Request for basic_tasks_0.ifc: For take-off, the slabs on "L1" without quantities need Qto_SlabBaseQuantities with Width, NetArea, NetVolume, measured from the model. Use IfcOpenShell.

First a look at what the model holds.

```python
import ifcopenshell
import ifcopenshell.util.element
import ifcopenshell.util.unit

model = ifcopenshell.open("basic_tasks_0.ifc")
print(model.schema)
for unit_type in ("LENGTHUNIT", "AREAUNIT", "VOLUMEUNIT"):
    print(unit_type, ifcopenshell.util.unit.calculate_unit_scale(model, unit_type))
storey = next(s for s in model.by_type("IfcBuildingStorey") if s.Name == "L1")
slabs = [e for e in ifcopenshell.util.element.get_decomposition(storey) if e.is_a("IfcSlab")]
for e in sorted(slabs, key=lambda e: e.id()):
    print(e.id(), e.is_a(), e.Name, list(ifcopenshell.util.element.get_psets(e, qtos_only=True)), sep=" | ")
```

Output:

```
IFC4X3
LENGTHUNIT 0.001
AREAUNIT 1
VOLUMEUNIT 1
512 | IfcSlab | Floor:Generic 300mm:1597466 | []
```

```python
import ifcopenshell
import ifcopenshell.api.pset
import ifcopenshell.geom
import ifcopenshell.util.element
import ifcopenshell.util.shape
import ifcopenshell.util.unit

model = ifcopenshell.open("basic_tasks_0.ifc")
unit_scale = ifcopenshell.util.unit.calculate_unit_scale(model)
area_scale = ifcopenshell.util.unit.calculate_unit_scale(model, "AREAUNIT")
volume_scale = ifcopenshell.util.unit.calculate_unit_scale(model, "VOLUMEUNIT")
settings = ifcopenshell.geom.settings()

storey = next(s for s in model.by_type("IfcBuildingStorey") if s.Name == "L1")
slabs = [e for e in ifcopenshell.util.element.get_decomposition(storey) if e.is_a("IfcSlab")]

for e in sorted(slabs, key=lambda e: e.id()):
    if ifcopenshell.util.element.get_psets(e, qtos_only=True, should_inherit=False):
        continue
    # Geometry comes back in metres, in the element's own axes.
    shape = ifcopenshell.geom.create_shape(settings, e)
    values = {
        "Width": ifcopenshell.util.shape.get_z(shape.geometry) / unit_scale,
        "NetArea": ifcopenshell.util.shape.get_footprint_area(shape.geometry) / area_scale,
        "NetVolume": ifcopenshell.util.shape.get_volume(shape.geometry) / volume_scale,
    }
    qto = ifcopenshell.api.pset.add_qto(model, product=e, name="Qto_SlabBaseQuantities")
    ifcopenshell.api.pset.edit_qto(model, qto=qto, properties=values)
    print(e.id(), {k: round(v, 3) for k, v in values.items()})

model.write("basic_tasks_0-out.ifc")
```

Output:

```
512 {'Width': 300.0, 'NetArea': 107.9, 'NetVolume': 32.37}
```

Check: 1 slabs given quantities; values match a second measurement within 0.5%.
